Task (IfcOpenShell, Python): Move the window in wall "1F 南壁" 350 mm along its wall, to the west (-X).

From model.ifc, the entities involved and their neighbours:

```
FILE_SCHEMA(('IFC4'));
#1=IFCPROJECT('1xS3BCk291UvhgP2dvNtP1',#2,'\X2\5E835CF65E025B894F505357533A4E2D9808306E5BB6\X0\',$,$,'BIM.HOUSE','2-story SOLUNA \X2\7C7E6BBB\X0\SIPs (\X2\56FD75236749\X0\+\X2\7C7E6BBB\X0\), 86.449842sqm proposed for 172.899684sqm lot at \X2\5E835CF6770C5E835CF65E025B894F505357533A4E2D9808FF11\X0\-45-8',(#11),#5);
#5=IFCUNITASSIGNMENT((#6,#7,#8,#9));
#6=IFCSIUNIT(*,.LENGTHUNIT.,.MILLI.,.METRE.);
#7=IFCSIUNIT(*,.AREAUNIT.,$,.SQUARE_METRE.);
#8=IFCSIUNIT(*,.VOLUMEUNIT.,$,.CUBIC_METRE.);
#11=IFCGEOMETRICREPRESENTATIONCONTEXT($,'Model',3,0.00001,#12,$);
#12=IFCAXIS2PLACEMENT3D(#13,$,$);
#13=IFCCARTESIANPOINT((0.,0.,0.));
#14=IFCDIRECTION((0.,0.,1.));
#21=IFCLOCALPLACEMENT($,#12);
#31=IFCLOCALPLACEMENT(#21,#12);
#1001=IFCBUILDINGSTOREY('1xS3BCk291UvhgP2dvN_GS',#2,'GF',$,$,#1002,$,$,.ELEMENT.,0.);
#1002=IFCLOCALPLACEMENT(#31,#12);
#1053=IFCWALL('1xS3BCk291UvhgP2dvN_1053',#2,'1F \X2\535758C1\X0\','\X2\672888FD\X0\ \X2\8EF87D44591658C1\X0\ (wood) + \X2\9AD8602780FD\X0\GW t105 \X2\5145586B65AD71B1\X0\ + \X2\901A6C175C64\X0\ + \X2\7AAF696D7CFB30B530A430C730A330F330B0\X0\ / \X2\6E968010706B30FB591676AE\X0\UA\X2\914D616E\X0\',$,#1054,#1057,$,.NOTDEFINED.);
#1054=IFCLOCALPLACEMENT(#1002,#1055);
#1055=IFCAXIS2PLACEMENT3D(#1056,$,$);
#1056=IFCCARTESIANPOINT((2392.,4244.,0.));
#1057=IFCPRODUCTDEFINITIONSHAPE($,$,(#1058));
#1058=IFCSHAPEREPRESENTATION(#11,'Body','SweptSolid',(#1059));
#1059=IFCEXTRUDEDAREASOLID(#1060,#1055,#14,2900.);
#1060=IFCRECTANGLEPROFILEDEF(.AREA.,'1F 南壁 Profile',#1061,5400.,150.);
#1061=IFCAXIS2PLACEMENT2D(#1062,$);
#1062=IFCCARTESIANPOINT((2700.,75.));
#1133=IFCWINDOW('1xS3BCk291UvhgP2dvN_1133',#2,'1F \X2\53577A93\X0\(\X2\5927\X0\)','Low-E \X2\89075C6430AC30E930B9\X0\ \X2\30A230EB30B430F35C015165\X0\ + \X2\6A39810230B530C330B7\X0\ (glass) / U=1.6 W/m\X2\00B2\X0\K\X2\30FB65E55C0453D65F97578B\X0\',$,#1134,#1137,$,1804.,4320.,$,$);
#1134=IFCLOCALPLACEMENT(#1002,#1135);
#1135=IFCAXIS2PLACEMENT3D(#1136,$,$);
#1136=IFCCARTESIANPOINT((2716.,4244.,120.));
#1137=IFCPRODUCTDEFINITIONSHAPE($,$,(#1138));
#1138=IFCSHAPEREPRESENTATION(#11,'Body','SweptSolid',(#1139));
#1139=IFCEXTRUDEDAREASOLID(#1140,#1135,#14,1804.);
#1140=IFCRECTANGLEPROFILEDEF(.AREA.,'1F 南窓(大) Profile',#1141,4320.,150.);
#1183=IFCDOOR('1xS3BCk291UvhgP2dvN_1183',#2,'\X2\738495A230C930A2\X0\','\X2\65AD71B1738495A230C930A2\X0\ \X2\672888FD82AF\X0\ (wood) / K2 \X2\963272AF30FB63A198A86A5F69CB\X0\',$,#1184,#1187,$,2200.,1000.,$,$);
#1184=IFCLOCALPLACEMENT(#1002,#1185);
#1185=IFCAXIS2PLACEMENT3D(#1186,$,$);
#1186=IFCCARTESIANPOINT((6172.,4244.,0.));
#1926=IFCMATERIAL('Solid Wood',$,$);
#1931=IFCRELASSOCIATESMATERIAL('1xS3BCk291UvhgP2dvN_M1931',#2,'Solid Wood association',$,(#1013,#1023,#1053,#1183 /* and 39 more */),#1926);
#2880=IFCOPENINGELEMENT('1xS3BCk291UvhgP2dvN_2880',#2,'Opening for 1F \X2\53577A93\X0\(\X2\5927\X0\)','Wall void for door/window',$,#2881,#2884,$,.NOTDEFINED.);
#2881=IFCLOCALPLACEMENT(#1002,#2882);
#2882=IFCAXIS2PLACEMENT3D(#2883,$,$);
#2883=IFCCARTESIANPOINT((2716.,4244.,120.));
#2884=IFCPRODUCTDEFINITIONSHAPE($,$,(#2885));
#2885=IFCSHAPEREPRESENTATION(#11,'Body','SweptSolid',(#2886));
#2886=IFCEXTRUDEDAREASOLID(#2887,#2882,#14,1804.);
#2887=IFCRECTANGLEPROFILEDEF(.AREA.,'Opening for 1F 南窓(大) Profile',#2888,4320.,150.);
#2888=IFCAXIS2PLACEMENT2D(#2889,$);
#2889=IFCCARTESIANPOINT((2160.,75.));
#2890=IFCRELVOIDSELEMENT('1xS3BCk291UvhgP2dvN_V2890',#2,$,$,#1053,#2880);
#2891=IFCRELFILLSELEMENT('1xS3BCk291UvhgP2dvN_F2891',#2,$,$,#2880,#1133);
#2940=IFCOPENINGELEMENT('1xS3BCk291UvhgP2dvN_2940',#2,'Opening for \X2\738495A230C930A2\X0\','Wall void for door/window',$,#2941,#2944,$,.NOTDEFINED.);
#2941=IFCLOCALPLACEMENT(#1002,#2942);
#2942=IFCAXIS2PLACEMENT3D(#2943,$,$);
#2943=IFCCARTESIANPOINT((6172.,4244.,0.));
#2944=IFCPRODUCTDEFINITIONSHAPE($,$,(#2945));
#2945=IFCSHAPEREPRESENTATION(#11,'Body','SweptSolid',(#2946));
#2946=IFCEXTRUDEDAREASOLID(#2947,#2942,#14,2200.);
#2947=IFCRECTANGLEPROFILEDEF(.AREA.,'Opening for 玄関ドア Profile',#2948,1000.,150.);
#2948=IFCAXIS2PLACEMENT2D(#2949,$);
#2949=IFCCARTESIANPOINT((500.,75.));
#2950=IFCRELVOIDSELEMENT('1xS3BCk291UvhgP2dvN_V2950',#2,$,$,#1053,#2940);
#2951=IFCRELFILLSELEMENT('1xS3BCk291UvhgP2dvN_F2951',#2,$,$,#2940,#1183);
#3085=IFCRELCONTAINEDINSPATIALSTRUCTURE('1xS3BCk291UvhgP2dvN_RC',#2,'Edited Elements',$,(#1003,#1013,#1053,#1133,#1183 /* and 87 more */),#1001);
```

```python
import ifcopenshell
import ifcopenshell.api.geometry
import ifcopenshell.util.placement
import ifcopenshell.util.unit

model = ifcopenshell.open("model.ifc")
unit_scale = ifcopenshell.util.unit.calculate_unit_scale(model)

window = model.by_guid("1xS3BCk291UvhgP2dvN_1133")
opening = window.FillsVoids[0].RelatingOpeningElement
wall = opening.VoidsElements[0].RelatingBuildingElement

wall_matrix = ifcopenshell.util.placement.get_local_placement(wall.ObjectPlacement)
shift = wall_matrix[:3, 0] * -0.35 / unit_scale
before = ifcopenshell.util.placement.get_local_placement(window.ObjectPlacement)[:3, 3].copy()

# The window is not placed relative to its opening, so move both.
for product in (opening, window):
    matrix = ifcopenshell.util.placement.get_local_placement(product.ObjectPlacement)
    matrix[:3, 3] += shift
    ifcopenshell.api.geometry.edit_object_placement(model, product=product, matrix=matrix, is_si=False)

after = ifcopenshell.util.placement.get_local_placement(window.ObjectPlacement)[:3, 3]
print("window moved by", (after - before).round(3) + 0.0)

model.write("model_updated.ifc")
```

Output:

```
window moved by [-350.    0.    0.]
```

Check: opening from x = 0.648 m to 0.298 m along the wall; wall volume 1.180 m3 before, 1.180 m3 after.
